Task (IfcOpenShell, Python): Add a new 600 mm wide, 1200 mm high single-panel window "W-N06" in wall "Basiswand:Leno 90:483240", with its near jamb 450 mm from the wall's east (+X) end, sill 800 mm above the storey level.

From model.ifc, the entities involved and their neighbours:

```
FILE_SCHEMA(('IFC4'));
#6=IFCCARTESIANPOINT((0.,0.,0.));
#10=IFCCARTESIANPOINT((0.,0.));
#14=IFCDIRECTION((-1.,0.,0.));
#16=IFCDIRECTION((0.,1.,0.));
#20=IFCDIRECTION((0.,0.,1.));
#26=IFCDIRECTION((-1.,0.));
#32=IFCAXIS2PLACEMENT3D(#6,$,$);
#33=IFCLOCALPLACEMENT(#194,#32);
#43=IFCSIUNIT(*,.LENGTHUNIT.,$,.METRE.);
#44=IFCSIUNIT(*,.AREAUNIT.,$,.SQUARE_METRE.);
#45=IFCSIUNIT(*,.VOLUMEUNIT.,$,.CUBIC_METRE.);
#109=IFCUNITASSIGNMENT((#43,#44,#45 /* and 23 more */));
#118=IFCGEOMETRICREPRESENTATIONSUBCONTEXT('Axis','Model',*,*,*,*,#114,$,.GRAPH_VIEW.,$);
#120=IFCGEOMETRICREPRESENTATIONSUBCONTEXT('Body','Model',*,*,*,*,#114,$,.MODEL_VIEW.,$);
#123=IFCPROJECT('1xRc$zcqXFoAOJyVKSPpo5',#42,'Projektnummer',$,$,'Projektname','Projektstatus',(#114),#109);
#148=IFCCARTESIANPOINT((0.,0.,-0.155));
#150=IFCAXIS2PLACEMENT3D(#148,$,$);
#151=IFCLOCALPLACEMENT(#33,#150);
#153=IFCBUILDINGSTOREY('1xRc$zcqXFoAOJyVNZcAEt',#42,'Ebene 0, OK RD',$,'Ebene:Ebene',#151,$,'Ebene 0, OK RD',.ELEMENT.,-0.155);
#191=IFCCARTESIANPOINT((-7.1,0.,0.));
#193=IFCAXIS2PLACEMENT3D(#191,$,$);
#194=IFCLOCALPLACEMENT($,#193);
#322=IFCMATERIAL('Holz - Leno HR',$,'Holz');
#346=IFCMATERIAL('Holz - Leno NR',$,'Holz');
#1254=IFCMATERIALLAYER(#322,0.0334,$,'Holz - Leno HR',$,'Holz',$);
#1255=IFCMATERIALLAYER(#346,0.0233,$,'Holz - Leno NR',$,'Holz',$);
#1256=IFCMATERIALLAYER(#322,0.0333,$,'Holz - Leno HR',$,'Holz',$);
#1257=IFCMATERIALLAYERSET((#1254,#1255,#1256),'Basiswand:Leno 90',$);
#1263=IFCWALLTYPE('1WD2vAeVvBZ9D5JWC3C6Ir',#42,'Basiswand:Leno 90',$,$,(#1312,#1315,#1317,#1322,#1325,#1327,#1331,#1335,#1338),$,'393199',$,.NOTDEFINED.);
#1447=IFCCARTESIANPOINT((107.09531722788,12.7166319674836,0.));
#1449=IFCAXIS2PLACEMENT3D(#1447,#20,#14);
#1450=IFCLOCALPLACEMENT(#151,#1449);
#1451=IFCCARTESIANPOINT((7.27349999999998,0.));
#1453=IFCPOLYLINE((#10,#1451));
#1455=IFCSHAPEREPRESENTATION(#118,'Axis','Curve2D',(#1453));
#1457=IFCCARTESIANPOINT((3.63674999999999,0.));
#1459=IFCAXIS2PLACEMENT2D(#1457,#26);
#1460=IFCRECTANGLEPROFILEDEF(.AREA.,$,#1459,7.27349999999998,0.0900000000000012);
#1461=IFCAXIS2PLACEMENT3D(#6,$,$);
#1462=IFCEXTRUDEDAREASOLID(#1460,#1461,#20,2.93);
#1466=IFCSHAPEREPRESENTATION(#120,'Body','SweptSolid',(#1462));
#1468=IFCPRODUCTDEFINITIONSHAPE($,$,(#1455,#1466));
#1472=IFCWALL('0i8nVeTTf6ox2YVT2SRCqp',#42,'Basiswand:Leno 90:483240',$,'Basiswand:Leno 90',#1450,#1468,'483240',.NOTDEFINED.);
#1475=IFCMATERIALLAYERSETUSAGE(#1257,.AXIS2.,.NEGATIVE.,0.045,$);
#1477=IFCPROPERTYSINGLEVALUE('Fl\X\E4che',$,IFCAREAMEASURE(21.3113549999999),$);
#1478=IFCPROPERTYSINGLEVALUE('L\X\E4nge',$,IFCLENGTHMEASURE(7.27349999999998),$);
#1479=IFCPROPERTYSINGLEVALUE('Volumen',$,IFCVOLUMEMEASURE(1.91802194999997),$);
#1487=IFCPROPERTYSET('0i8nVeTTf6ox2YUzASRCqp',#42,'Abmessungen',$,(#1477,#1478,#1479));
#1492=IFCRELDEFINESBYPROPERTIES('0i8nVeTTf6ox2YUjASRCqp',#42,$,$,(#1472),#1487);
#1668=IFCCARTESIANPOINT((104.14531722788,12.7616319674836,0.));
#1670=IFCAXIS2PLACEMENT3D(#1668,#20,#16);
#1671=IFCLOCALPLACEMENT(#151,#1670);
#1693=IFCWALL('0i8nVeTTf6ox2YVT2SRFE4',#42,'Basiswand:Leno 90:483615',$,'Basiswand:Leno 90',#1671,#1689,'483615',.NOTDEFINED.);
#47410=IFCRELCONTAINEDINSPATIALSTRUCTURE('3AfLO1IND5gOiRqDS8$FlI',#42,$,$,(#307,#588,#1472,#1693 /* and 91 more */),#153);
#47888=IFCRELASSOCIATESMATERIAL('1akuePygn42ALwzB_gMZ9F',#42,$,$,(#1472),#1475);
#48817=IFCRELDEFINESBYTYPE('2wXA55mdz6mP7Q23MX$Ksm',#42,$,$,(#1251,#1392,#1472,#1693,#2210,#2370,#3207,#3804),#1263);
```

```python
import numpy as np
import ifcopenshell
import ifcopenshell.api.feature
import ifcopenshell.api.geometry
import ifcopenshell.api.pset
import ifcopenshell.api.root
import ifcopenshell.api.spatial
import ifcopenshell.geom
import ifcopenshell.util.element
import ifcopenshell.util.placement
import ifcopenshell.util.representation
import ifcopenshell.util.shape
import ifcopenshell.util.unit

model = ifcopenshell.open("model.ifc")
unit_scale = ifcopenshell.util.unit.calculate_unit_scale(model)
area_scale = ifcopenshell.util.unit.calculate_unit_scale(model, "AREAUNIT")
volume_scale = ifcopenshell.util.unit.calculate_unit_scale(model, "VOLUMEUNIT")
settings = ifcopenshell.geom.settings()


def volume(element):
    """Net volume in cubic metres, openings subtracted."""
    shape = ifcopenshell.geom.create_shape(settings, element)
    return ifcopenshell.util.shape.get_volume(shape.geometry)


wall = model.by_guid("0i8nVeTTf6ox2YVT2SRCqp")
storey = ifcopenshell.util.element.get_container(wall, ifc_class="IfcBuildingStorey")
context = ifcopenshell.util.representation.get_context(model, "Model", "Body", "MODEL_VIEW")
before = volume(wall)

width, height, from_end, sill = 0.6, 1.2, 0.45, 0.8  # metres

# The wall runs along its own X axis, and the end named is its -X end.
wall_shape = ifcopenshell.geom.create_shape(settings, wall)
x, y, z = ifcopenshell.util.shape.get_vertices(wall_shape.geometry).T
start = x.min() + from_end
face, thickness = float(y.min()), float(y.max() - y.min())
wall_matrix = ifcopenshell.util.placement.get_local_placement(wall.ObjectPlacement)
level = ifcopenshell.util.placement.get_local_placement(storey.ObjectPlacement)[2, 3]


def in_wall(x, y):
    """Placement at x, y metres in the wall's axes, at sill height."""
    matrix = wall_matrix.copy()
    matrix[:, 3] = wall_matrix @ np.array([x / unit_scale, y / unit_scale, 0.0, 1.0])
    matrix[2, 3] = level + sill / unit_scale
    return matrix


# Opening: a box that overshoots both wall faces by 50 mm.
opening = ifcopenshell.api.root.create_entity(model, ifc_class="IfcOpeningElement", predefined_type="OPENING")
box = ifcopenshell.api.geometry.add_wall_representation(
    model, context=context, length=width, height=height, thickness=thickness + 0.1
)
ifcopenshell.api.geometry.assign_representation(model, product=opening, representation=box)
ifcopenshell.api.geometry.edit_object_placement(model, product=opening, matrix=in_wall(start, face - 0.05), is_si=False)
ifcopenshell.api.feature.add_feature(model, feature=opening, element=wall)

window = ifcopenshell.api.root.create_entity(model, ifc_class="IfcWindow", name="W-N06", predefined_type="WINDOW")
window.OverallWidth, window.OverallHeight = width / unit_scale, height / unit_scale
window.PartitioningType = "SINGLE_PANEL"
body = ifcopenshell.api.geometry.add_window_representation(
    model,
    context=context,
    overall_width=window.OverallWidth,
    overall_height=window.OverallHeight,
    partition_type="SINGLE_PANEL",
)
ifcopenshell.api.geometry.assign_representation(model, product=window, representation=body)
ifcopenshell.api.spatial.assign_container(model, products=[window], relating_structure=storey)
ifcopenshell.api.feature.add_filling(model, opening=opening, element=window)

# Centre the window in the wall's thickness.
ifcopenshell.api.geometry.edit_object_placement(model, product=window, matrix=in_wall(start, face), is_si=False)
window_shape = ifcopenshell.geom.create_shape(settings, window)
depth = ifcopenshell.util.shape.get_vertices(window_shape.geometry)[:, 1]
offset = face + thickness / 2 - (depth.min() + depth.max()) / 2
ifcopenshell.api.geometry.edit_object_placement(model, product=window, matrix=in_wall(start, offset), is_si=False)

after = volume(wall)

# Update the wall's stored quantities.
pset = model.by_id(ifcopenshell.util.element.get_pset(wall, "Abmessungen", should_inherit=False)["id"])
ifcopenshell.api.pset.edit_pset(model, pset=pset, properties={
    "Fläche": model.create_entity("IfcAreaMeasure", after / thickness / area_scale),
    "Volumen": model.create_entity("IfcVolumeMeasure", after / volume_scale),
})

print(f"wall volume {before:.3f} -> {after:.3f} m3")

model.write("model-out.ifc")
```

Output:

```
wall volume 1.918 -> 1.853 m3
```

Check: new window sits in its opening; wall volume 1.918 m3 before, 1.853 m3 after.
